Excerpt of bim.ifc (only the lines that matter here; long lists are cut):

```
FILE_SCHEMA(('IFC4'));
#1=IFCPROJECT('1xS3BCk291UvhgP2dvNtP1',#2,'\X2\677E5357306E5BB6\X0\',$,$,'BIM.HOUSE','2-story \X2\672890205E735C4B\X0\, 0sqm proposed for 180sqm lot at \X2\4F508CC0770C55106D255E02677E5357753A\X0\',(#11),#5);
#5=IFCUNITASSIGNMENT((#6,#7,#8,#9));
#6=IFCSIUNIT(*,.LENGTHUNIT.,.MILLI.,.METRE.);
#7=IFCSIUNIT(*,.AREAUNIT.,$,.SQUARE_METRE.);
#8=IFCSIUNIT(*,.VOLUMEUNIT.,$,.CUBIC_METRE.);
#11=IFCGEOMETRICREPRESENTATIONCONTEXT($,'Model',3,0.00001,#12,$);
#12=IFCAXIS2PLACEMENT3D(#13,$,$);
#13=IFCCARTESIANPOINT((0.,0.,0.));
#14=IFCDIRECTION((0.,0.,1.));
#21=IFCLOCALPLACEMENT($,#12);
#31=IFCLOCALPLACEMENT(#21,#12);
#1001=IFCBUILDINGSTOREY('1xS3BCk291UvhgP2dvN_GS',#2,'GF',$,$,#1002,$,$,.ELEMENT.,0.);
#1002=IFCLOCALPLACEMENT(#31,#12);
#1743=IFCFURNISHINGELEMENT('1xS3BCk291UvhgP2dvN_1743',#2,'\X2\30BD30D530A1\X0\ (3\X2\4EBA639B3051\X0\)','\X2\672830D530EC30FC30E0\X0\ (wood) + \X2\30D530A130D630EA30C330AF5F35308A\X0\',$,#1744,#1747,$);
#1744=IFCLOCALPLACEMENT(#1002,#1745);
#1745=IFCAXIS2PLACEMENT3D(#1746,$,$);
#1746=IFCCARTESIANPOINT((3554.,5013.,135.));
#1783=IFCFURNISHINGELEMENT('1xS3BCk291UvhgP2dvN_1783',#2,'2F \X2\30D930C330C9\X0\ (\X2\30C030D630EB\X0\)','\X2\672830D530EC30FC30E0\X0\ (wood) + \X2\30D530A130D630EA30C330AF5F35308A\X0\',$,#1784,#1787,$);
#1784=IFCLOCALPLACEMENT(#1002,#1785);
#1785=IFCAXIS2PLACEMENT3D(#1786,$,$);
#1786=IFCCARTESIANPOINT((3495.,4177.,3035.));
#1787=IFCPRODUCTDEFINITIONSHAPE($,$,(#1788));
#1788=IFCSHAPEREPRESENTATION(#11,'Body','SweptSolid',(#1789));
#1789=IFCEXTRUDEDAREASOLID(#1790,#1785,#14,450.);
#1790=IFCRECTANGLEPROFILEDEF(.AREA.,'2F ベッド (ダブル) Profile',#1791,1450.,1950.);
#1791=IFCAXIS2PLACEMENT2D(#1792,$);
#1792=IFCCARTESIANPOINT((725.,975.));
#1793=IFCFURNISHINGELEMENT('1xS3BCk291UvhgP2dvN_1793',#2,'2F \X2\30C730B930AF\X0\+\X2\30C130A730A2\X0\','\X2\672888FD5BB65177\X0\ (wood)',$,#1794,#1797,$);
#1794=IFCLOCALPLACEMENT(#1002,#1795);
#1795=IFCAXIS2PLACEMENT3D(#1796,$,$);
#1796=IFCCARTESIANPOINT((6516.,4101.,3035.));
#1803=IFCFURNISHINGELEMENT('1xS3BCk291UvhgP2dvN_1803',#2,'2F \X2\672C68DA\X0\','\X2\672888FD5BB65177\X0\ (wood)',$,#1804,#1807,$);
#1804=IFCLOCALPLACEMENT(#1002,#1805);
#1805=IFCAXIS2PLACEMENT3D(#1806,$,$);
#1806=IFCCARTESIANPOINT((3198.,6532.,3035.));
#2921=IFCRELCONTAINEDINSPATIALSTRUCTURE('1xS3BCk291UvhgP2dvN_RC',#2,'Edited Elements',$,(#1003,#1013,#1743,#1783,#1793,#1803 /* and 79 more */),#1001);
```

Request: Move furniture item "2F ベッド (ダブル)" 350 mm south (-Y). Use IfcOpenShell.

```python
import ifcopenshell
import ifcopenshell.api.geometry
import ifcopenshell.util.placement
import ifcopenshell.util.unit

model = ifcopenshell.open("bim.ifc")
unit_scale = ifcopenshell.util.unit.calculate_unit_scale(model)

item = model.by_guid("1xS3BCk291UvhgP2dvN_1783")
matrix = ifcopenshell.util.placement.get_local_placement(item.ObjectPlacement)
matrix[1, 3] -= 0.35 / unit_scale
ifcopenshell.api.geometry.edit_object_placement(model, product=item, matrix=matrix, is_si=False)

print(ifcopenshell.util.placement.get_local_placement(item.ObjectPlacement).round(3) + 0.0)

model.write("bim_rev.ifc")
```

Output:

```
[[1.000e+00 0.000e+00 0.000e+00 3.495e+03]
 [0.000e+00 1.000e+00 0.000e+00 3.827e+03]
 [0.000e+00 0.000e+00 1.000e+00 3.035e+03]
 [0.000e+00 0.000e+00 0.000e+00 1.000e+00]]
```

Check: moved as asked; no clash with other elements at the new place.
